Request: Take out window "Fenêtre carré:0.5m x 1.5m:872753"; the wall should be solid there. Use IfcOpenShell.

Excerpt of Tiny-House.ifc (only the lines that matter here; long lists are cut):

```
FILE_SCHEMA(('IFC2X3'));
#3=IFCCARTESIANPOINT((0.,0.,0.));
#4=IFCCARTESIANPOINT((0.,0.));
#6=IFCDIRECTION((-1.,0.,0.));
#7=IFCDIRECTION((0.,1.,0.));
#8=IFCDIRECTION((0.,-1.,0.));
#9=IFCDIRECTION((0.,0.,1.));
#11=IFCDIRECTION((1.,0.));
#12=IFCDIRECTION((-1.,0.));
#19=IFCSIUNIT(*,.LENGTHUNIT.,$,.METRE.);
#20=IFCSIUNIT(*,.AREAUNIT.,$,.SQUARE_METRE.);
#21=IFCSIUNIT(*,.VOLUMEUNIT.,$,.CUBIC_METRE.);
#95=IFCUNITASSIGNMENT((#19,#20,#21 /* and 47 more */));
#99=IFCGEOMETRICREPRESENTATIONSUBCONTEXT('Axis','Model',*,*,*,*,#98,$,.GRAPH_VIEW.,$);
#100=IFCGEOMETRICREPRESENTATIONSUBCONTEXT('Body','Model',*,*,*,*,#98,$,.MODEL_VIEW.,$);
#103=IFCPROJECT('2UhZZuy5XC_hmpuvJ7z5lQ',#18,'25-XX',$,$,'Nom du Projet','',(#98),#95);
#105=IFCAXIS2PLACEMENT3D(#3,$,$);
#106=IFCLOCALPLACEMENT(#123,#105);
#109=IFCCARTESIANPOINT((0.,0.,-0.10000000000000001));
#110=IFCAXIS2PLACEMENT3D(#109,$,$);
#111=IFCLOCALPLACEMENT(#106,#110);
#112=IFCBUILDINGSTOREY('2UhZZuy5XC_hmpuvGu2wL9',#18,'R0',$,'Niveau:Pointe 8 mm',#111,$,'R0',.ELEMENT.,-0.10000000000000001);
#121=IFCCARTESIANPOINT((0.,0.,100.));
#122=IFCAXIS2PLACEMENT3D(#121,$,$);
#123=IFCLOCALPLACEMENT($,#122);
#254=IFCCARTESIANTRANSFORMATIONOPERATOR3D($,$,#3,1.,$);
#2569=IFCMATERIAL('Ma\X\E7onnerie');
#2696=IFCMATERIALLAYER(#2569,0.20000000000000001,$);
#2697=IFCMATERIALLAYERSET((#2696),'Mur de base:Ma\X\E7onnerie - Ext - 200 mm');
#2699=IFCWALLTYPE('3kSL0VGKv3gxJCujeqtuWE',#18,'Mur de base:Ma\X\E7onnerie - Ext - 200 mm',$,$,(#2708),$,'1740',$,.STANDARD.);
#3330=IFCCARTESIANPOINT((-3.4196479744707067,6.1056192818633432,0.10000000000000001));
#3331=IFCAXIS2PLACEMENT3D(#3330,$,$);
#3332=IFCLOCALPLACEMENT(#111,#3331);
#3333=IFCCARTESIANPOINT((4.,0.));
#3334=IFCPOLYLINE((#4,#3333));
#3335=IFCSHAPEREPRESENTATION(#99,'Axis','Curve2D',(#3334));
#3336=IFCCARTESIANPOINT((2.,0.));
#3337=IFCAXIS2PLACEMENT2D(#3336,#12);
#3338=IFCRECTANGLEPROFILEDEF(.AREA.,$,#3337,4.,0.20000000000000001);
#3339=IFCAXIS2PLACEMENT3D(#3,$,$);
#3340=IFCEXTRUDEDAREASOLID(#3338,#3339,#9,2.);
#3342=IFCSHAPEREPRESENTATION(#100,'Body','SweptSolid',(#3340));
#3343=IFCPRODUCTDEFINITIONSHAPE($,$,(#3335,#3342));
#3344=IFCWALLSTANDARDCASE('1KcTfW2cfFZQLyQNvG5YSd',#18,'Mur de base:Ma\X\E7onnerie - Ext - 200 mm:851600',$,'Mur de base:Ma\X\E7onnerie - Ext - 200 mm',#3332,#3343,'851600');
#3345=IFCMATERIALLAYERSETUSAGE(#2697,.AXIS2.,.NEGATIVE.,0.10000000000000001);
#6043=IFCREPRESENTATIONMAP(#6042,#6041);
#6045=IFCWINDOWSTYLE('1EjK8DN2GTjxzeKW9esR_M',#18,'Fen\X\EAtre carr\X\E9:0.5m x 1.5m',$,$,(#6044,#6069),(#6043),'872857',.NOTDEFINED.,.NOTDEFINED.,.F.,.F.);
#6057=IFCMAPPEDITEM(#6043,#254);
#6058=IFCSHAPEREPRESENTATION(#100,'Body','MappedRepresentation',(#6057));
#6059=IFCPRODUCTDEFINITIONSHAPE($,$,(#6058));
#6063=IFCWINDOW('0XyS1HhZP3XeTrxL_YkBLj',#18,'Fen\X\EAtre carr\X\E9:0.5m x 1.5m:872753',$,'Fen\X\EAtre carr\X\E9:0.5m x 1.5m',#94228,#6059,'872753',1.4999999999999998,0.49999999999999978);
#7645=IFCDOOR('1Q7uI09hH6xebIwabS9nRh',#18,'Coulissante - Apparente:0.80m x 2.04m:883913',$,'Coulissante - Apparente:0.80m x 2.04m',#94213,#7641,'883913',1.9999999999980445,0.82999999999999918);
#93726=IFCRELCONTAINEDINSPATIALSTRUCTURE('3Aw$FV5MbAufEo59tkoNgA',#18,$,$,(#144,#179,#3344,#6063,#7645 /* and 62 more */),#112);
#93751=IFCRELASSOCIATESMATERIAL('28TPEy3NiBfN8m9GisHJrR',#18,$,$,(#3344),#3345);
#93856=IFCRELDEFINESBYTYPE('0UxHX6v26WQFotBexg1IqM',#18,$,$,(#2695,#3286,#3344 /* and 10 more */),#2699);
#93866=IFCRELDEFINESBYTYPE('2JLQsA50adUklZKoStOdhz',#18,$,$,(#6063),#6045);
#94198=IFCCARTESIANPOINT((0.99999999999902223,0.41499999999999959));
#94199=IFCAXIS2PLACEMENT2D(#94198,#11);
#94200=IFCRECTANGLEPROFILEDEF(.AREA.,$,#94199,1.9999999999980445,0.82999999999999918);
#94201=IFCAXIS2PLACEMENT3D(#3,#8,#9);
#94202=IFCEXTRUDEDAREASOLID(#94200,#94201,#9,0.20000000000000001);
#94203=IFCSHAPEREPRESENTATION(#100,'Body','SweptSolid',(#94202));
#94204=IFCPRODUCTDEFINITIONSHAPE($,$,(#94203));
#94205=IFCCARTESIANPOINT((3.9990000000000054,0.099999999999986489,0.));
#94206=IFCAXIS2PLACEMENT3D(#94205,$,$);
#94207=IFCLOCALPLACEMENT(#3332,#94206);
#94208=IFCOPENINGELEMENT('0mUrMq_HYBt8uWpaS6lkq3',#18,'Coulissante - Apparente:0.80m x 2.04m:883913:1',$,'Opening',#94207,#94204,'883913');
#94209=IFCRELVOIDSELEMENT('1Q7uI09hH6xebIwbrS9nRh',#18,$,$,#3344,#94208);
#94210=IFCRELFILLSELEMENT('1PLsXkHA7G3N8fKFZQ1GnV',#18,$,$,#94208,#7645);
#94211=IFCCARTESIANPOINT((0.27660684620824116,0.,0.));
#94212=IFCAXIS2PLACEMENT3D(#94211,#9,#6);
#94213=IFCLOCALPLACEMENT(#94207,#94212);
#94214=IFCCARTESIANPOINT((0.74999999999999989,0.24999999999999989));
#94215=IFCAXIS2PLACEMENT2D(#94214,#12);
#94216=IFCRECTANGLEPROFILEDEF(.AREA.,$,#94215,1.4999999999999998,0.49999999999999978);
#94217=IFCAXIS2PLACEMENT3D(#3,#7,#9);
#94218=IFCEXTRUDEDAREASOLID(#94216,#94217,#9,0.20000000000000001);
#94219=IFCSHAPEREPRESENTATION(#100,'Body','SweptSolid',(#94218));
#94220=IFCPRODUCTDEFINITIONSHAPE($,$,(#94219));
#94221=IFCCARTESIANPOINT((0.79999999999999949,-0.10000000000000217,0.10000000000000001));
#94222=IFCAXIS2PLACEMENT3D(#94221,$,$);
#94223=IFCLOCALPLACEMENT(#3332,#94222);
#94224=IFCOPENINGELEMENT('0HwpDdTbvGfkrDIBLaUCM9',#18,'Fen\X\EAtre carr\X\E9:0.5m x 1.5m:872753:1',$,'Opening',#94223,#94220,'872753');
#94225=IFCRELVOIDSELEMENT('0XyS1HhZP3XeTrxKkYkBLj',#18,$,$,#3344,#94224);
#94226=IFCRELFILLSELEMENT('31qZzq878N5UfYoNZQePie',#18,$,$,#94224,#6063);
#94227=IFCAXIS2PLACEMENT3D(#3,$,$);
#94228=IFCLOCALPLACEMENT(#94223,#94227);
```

```python
import ifcopenshell
import ifcopenshell.api.feature
import ifcopenshell.api.root
import ifcopenshell.geom
import ifcopenshell.util.shape

model = ifcopenshell.open("Tiny-House.ifc")
settings = ifcopenshell.geom.settings()


def volume(element):
    """Net volume in cubic metres, openings subtracted."""
    shape = ifcopenshell.geom.create_shape(settings, element)
    return ifcopenshell.util.shape.get_volume(shape.geometry)


window = model.by_id(6063)
opening = window.FillsVoids[0].RelatingOpeningElement
wall = opening.VoidsElements[0].RelatingBuildingElement
before = volume(wall)

ifcopenshell.api.root.remove_product(model, product=window)
ifcopenshell.api.feature.remove_feature(model, feature=opening)

after = volume(wall)

print(f"wall volume {before:.3f} -> {after:.3f} m3")

model.write("Tiny-House_edited.ifc")
```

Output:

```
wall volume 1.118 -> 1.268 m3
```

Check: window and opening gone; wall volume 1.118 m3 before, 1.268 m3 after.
